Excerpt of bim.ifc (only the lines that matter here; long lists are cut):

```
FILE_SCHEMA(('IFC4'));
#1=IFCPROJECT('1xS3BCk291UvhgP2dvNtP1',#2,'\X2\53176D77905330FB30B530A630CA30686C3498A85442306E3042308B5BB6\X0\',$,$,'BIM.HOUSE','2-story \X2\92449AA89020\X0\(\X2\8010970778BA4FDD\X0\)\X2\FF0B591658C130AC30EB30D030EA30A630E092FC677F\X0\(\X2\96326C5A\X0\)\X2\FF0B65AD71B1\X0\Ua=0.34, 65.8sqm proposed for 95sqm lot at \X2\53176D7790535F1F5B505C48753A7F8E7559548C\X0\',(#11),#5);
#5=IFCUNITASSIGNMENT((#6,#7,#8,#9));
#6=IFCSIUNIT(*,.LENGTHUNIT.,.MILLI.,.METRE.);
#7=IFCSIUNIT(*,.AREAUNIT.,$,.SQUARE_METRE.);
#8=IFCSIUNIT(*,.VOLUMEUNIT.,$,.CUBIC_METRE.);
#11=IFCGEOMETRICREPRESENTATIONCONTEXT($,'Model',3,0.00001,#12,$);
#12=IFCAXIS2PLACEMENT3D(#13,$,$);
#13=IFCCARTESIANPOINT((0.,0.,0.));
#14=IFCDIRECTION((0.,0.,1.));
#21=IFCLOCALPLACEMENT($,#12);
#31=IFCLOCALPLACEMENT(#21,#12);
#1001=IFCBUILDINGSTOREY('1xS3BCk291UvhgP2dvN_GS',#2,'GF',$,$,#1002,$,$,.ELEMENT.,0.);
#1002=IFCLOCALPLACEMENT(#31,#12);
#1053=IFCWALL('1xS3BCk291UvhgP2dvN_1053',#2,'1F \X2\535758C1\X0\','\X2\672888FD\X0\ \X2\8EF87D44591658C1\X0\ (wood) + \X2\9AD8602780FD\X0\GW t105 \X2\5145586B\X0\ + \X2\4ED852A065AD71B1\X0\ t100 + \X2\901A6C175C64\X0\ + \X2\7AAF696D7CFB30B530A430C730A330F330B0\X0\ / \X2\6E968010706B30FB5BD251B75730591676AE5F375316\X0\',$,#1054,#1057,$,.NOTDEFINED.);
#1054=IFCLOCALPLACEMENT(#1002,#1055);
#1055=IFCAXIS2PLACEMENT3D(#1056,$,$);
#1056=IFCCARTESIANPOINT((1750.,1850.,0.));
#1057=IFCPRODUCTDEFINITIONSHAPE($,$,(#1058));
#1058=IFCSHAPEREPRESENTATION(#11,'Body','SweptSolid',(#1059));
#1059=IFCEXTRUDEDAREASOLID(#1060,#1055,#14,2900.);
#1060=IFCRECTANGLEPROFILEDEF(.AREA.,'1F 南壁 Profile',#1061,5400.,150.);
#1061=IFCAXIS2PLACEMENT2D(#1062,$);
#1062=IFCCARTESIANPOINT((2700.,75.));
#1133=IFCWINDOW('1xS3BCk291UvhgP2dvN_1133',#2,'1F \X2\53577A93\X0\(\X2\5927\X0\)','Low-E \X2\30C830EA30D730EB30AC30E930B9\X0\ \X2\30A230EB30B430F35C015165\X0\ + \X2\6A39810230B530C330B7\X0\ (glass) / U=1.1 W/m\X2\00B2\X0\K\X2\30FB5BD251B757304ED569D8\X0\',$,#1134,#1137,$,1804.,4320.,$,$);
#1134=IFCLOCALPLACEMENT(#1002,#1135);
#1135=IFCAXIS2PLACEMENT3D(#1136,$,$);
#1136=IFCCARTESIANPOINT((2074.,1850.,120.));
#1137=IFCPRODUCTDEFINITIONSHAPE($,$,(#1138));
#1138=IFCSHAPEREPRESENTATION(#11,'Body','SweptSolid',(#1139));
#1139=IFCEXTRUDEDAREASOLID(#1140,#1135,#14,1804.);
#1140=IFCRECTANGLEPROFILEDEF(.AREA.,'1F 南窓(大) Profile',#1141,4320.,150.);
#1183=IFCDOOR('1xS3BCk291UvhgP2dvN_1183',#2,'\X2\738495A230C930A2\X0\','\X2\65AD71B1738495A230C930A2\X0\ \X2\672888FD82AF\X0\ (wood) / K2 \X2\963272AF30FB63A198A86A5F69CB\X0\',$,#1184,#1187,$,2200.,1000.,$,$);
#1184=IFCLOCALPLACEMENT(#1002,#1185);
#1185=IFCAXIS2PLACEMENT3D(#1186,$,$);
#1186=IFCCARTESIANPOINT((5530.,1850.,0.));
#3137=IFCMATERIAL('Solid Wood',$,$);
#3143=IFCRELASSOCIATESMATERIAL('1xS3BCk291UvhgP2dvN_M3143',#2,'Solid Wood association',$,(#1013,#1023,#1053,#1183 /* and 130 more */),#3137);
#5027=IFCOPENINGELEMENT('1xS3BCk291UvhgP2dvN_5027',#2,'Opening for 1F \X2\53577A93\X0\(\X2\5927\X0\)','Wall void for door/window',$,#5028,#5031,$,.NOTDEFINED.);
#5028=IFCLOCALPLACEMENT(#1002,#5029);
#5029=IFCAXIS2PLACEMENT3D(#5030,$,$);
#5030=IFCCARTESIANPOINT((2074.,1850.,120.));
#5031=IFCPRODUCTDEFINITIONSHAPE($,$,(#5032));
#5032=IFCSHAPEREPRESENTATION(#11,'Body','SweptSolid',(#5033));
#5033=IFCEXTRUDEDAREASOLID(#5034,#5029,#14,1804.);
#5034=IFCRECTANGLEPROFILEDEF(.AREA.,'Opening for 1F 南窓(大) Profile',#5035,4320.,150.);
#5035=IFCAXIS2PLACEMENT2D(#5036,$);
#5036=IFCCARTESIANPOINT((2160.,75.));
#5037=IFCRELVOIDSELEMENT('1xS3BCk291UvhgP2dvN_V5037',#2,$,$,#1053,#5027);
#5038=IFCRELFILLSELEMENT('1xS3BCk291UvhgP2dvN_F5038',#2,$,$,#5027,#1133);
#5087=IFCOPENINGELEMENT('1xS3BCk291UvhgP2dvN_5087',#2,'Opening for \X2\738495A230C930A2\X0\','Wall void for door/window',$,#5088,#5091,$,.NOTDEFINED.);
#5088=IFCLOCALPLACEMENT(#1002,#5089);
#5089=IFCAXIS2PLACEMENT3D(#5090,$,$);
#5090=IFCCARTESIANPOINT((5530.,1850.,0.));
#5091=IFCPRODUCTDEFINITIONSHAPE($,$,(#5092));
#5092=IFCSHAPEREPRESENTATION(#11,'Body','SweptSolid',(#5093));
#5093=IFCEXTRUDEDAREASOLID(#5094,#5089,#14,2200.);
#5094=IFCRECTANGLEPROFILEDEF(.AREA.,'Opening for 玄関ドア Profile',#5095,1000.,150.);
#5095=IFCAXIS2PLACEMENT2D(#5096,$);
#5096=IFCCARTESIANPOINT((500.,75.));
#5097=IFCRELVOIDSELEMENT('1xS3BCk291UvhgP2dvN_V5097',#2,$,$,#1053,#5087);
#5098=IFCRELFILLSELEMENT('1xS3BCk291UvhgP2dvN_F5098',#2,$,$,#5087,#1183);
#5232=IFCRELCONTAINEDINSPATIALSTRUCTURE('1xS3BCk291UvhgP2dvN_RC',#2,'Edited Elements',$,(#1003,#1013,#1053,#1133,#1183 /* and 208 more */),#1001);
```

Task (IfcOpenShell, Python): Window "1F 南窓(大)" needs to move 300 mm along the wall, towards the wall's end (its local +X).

```python
import ifcopenshell
import ifcopenshell.api.geometry
import ifcopenshell.util.placement

model = ifcopenshell.open("bim.ifc")

window = model.by_guid("1xS3BCk291UvhgP2dvN_1133")
opening = window.FillsVoids[0].RelatingOpeningElement
wall = opening.VoidsElements[0].RelatingBuildingElement

wall_matrix = ifcopenshell.util.placement.get_local_placement(wall.ObjectPlacement)
shift = wall_matrix[:3, 0] * 300.0
before = ifcopenshell.util.placement.get_local_placement(window.ObjectPlacement)[:3, 3].copy()

# The window is not placed relative to its opening, so move both.
for product in (opening, window):
    matrix = ifcopenshell.util.placement.get_local_placement(product.ObjectPlacement)
    matrix[:3, 3] += shift
    ifcopenshell.api.geometry.edit_object_placement(model, product=product, matrix=matrix, is_si=False)

after = ifcopenshell.util.placement.get_local_placement(window.ObjectPlacement)[:3, 3]
print("window moved by", (after - before).round(3) + 0.0)

model.write("bim_v2.ifc")
```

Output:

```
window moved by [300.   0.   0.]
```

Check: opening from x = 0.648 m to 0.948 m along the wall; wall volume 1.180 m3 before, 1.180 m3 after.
